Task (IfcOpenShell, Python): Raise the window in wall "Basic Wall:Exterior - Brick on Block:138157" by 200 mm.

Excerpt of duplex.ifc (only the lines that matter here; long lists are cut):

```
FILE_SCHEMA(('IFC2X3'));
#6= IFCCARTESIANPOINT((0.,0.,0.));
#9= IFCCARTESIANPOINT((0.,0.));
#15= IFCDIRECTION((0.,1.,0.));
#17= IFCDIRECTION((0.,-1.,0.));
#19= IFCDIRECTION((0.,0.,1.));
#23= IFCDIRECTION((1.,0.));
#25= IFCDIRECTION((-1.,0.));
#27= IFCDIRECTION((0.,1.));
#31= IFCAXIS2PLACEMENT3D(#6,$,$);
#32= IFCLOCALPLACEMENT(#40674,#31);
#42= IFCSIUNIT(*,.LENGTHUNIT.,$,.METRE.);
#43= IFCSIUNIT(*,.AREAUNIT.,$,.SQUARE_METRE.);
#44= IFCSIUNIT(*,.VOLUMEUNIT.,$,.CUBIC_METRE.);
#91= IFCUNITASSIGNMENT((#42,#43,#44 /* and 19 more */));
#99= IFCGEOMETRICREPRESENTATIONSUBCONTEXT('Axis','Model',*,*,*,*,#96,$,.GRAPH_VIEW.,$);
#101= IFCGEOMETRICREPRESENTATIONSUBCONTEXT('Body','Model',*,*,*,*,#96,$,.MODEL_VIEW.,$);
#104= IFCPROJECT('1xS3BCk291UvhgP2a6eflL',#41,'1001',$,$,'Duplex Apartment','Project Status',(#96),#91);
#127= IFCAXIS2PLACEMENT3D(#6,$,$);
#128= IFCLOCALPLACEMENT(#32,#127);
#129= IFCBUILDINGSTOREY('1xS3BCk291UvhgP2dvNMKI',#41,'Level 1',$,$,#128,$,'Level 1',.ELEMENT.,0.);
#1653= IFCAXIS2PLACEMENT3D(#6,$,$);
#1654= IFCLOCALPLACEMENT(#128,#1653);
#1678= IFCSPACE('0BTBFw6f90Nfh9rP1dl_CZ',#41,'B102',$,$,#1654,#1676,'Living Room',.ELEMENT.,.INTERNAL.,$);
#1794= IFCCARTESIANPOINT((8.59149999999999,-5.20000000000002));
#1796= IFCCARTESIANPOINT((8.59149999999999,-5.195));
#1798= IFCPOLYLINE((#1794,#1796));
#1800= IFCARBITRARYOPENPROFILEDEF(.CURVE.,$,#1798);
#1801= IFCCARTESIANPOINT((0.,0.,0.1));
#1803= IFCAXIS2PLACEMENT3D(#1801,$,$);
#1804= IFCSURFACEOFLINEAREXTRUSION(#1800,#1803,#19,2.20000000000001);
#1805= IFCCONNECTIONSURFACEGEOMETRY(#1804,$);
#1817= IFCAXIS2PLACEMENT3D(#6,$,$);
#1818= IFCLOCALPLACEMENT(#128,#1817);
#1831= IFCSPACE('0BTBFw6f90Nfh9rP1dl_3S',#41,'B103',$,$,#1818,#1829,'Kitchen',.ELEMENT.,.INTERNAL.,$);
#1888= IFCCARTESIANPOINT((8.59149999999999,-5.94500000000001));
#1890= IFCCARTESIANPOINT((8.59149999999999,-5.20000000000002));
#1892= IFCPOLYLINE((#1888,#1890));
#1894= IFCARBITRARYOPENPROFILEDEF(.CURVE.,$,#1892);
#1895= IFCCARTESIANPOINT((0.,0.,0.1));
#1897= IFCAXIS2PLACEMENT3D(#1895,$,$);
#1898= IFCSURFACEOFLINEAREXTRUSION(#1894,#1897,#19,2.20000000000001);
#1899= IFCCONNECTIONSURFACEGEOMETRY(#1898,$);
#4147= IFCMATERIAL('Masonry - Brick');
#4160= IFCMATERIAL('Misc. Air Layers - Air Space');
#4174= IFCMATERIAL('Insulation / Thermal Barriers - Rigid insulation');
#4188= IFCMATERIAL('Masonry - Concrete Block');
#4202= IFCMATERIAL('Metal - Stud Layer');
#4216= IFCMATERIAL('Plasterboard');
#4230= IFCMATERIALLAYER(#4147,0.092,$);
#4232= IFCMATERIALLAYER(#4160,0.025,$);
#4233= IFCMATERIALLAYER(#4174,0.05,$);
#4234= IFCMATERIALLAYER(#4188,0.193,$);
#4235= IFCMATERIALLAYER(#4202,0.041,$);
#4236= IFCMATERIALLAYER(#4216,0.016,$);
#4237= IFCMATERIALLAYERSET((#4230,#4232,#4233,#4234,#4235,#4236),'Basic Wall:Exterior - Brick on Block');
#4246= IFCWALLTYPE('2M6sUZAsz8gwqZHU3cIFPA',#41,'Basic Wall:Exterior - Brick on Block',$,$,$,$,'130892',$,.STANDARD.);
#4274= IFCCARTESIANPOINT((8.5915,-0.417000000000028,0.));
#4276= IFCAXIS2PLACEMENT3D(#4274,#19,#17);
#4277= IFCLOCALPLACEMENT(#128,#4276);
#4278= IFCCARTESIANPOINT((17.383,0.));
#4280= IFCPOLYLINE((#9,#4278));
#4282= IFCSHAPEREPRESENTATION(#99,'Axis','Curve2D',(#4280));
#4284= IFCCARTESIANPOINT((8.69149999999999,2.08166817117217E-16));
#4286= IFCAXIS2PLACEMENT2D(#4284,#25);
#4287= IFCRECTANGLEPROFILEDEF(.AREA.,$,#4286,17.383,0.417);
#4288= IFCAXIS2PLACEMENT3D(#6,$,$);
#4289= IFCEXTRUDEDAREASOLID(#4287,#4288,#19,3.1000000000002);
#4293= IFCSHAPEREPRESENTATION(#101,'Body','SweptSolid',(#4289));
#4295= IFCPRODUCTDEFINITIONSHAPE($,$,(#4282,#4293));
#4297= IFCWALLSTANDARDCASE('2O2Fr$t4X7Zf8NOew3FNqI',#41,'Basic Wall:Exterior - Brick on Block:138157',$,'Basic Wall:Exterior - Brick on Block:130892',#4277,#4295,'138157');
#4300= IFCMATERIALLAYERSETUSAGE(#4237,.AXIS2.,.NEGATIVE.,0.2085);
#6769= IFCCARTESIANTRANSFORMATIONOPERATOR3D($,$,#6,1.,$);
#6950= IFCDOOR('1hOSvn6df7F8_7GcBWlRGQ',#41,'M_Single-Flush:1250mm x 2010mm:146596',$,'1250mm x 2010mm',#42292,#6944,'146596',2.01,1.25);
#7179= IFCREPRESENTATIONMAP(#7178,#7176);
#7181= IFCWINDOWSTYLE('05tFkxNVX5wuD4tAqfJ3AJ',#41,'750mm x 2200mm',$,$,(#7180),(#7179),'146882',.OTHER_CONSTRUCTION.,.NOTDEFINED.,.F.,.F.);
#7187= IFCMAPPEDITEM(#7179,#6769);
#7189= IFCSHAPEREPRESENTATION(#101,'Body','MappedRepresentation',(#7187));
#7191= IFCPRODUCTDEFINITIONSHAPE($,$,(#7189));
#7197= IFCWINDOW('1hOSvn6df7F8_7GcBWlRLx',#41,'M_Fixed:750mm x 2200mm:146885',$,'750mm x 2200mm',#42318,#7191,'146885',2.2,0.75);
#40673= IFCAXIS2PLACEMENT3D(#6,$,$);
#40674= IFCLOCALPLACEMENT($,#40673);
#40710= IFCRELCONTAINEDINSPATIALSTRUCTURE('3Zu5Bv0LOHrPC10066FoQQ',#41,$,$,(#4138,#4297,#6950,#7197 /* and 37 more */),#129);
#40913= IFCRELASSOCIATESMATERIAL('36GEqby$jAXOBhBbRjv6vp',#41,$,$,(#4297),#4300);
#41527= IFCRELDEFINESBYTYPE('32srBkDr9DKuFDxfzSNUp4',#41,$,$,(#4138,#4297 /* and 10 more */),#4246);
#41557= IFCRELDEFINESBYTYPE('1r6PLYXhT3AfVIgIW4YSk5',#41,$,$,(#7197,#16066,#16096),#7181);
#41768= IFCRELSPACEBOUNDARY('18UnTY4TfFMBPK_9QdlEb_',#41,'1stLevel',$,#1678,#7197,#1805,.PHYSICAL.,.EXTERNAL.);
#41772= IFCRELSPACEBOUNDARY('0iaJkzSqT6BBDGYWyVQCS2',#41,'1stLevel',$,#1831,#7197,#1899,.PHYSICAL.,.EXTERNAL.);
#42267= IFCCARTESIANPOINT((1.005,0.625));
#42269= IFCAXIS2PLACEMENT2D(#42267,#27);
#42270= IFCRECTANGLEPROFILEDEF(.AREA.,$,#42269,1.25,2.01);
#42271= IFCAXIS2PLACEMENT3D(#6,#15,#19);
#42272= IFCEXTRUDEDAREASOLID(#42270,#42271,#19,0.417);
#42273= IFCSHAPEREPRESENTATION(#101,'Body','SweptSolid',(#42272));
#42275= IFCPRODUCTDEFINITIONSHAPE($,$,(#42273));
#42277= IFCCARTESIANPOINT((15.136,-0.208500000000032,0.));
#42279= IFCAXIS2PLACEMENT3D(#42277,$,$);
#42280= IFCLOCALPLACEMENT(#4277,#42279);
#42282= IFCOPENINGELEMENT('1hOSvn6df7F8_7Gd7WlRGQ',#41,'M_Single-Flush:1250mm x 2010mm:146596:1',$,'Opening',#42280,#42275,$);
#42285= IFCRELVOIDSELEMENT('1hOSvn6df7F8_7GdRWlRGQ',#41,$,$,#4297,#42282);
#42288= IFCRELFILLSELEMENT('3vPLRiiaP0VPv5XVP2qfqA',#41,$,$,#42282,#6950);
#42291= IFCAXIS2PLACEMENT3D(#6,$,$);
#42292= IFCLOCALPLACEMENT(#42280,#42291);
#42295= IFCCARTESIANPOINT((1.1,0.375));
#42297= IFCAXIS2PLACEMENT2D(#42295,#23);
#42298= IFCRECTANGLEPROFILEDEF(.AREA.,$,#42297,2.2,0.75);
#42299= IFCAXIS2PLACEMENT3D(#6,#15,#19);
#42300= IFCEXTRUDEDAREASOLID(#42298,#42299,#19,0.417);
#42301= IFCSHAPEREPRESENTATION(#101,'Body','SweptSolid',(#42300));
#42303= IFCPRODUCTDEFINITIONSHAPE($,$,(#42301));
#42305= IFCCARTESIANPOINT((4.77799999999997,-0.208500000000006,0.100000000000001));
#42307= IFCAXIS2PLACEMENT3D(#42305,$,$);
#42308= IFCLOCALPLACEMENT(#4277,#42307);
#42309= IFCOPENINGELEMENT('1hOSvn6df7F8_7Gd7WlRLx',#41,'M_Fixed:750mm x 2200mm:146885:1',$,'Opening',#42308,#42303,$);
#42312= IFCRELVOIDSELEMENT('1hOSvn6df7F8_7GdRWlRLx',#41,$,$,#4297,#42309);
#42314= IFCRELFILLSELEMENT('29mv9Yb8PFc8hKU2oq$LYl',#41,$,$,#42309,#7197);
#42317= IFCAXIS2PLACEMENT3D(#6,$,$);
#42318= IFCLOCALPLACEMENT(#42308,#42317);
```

```python
import numpy as np
import ifcopenshell
import ifcopenshell.api.geometry
import ifcopenshell.util.placement
import ifcopenshell.util.unit

model = ifcopenshell.open("duplex.ifc")
unit_scale = ifcopenshell.util.unit.calculate_unit_scale(model)

window = model.by_guid("1hOSvn6df7F8_7GcBWlRLx")
opening = window.FillsVoids[0].RelatingOpeningElement
dz = 0.2 / unit_scale

shift = np.array([0.0, 0.0, dz])
# The window is placed relative to its opening, so it follows when the opening moves.
matrix = ifcopenshell.util.placement.get_local_placement(opening.ObjectPlacement)
matrix[:3, 3] += shift
ifcopenshell.api.geometry.edit_object_placement(
    model, product=opening, matrix=matrix, is_si=False, should_transform_children=True
)

# Space boundary surfaces are stored in each space's coordinates; move them too.
for rel in window.ProvidesBoundaries:
    if not rel.ConnectionGeometry:
        continue
    surface = rel.ConnectionGeometry.SurfaceOnRelatingElement
    space_matrix = ifcopenshell.util.placement.get_local_placement(rel.RelatingSpace.ObjectPlacement)
    point = np.array(surface.Position.Location.Coordinates) + space_matrix[:3, :3].T @ shift
    surface.Position = model.createIfcAxis2Placement3D(
        model.createIfcCartesianPoint(point.tolist()), surface.Position.Axis, surface.Position.RefDirection
    )

print(f"moved by {dz * unit_scale:+.3f} m")

model.write("duplex_edited.ifc")
```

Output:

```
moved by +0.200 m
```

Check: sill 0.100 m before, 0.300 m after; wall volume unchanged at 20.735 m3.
